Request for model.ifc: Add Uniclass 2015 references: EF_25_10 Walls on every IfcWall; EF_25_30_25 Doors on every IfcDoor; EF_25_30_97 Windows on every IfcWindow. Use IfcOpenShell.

First a look at what the model holds.

```python
import ifcopenshell

model = ifcopenshell.open("model.ifc")
print(model.schema)
print("classifications:", [c.Name for c in model.by_type("IfcClassification")])
for ifc_class in ("IfcDoor", "IfcRoof", "IfcStair", "IfcWall", "IfcWindow"):
    print(ifc_class, len(model.by_type(ifc_class)))
```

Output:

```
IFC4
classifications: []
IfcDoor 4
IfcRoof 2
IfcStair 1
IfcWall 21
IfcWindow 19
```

```python
import ifcopenshell
import ifcopenshell.api.classification

model = ifcopenshell.open("model.ifc")

system = ifcopenshell.api.classification.add_classification(model, classification="Uniclass 2015")

codes = {
    "IfcWall": ("EF_25_10", "Walls"),
    "IfcDoor": ("EF_25_30_25", "Doors"),
    "IfcWindow": ("EF_25_30_97", "Windows"),
}
for ifc_class, (code, name) in codes.items():
    products = model.by_type(ifc_class)
    ifcopenshell.api.classification.add_reference(
        model, products=products, classification=system, identification=code, name=name
    )
    print(code, len(products))

model.write("model_v2.ifc")
```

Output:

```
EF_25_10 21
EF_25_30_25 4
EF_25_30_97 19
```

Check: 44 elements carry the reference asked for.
